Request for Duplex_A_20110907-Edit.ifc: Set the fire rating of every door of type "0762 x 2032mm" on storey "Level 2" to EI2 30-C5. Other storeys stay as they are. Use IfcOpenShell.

First a look at what the model holds.

```python
import ifcopenshell
import ifcopenshell.util.element

model = ifcopenshell.open("Duplex_A_20110907-Edit.ifc")
print(model.schema)
storey = next(s for s in model.by_type("IfcBuildingStorey") if s.Name == "Level 2")
doors = [e for e in ifcopenshell.util.element.get_decomposition(storey) if e.is_a("IfcDoor")]
seen = {}
for e in doors:
    element_type = ifcopenshell.util.element.get_type(e)
    key = (element_type.Name if element_type != e and element_type else None, ifcopenshell.util.element.get_pset(e, "Pset_DoorCommon", "FireRating"))
    seen[key] = seen.get(key, 0) + 1
for (name, value), count in sorted(seen.items(), key=str):
    print(count, "x", name, "|", value)
```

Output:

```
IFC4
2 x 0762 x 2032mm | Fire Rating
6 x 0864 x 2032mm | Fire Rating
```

```python
import ifcopenshell
import ifcopenshell.api.pset
import ifcopenshell.util.element

model = ifcopenshell.open("Duplex_A_20110907-Edit.ifc")

storey = next(s for s in model.by_type("IfcBuildingStorey") if s.Name == "Level 2")
doors = [e for e in ifcopenshell.util.element.get_decomposition(storey) if e.is_a("IfcDoor")]

count = 0
for e in doors:
    element_type = ifcopenshell.util.element.get_type(e)
    if element_type in (None, e) or element_type.Name != "0762 x 2032mm":
        continue
    # add_pset returns the element's existing set when there is one.
    pset = ifcopenshell.api.pset.add_pset(model, product=e, name="Pset_DoorCommon")
    ifcopenshell.api.pset.edit_pset(model, pset=pset, properties={"FireRating": "EI2 30-C5"})
    count += 1

print(count, "doors updated")

model.write("Duplex_A_20110907-Edit_edited.ifc")
```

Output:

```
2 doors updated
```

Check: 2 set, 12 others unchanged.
